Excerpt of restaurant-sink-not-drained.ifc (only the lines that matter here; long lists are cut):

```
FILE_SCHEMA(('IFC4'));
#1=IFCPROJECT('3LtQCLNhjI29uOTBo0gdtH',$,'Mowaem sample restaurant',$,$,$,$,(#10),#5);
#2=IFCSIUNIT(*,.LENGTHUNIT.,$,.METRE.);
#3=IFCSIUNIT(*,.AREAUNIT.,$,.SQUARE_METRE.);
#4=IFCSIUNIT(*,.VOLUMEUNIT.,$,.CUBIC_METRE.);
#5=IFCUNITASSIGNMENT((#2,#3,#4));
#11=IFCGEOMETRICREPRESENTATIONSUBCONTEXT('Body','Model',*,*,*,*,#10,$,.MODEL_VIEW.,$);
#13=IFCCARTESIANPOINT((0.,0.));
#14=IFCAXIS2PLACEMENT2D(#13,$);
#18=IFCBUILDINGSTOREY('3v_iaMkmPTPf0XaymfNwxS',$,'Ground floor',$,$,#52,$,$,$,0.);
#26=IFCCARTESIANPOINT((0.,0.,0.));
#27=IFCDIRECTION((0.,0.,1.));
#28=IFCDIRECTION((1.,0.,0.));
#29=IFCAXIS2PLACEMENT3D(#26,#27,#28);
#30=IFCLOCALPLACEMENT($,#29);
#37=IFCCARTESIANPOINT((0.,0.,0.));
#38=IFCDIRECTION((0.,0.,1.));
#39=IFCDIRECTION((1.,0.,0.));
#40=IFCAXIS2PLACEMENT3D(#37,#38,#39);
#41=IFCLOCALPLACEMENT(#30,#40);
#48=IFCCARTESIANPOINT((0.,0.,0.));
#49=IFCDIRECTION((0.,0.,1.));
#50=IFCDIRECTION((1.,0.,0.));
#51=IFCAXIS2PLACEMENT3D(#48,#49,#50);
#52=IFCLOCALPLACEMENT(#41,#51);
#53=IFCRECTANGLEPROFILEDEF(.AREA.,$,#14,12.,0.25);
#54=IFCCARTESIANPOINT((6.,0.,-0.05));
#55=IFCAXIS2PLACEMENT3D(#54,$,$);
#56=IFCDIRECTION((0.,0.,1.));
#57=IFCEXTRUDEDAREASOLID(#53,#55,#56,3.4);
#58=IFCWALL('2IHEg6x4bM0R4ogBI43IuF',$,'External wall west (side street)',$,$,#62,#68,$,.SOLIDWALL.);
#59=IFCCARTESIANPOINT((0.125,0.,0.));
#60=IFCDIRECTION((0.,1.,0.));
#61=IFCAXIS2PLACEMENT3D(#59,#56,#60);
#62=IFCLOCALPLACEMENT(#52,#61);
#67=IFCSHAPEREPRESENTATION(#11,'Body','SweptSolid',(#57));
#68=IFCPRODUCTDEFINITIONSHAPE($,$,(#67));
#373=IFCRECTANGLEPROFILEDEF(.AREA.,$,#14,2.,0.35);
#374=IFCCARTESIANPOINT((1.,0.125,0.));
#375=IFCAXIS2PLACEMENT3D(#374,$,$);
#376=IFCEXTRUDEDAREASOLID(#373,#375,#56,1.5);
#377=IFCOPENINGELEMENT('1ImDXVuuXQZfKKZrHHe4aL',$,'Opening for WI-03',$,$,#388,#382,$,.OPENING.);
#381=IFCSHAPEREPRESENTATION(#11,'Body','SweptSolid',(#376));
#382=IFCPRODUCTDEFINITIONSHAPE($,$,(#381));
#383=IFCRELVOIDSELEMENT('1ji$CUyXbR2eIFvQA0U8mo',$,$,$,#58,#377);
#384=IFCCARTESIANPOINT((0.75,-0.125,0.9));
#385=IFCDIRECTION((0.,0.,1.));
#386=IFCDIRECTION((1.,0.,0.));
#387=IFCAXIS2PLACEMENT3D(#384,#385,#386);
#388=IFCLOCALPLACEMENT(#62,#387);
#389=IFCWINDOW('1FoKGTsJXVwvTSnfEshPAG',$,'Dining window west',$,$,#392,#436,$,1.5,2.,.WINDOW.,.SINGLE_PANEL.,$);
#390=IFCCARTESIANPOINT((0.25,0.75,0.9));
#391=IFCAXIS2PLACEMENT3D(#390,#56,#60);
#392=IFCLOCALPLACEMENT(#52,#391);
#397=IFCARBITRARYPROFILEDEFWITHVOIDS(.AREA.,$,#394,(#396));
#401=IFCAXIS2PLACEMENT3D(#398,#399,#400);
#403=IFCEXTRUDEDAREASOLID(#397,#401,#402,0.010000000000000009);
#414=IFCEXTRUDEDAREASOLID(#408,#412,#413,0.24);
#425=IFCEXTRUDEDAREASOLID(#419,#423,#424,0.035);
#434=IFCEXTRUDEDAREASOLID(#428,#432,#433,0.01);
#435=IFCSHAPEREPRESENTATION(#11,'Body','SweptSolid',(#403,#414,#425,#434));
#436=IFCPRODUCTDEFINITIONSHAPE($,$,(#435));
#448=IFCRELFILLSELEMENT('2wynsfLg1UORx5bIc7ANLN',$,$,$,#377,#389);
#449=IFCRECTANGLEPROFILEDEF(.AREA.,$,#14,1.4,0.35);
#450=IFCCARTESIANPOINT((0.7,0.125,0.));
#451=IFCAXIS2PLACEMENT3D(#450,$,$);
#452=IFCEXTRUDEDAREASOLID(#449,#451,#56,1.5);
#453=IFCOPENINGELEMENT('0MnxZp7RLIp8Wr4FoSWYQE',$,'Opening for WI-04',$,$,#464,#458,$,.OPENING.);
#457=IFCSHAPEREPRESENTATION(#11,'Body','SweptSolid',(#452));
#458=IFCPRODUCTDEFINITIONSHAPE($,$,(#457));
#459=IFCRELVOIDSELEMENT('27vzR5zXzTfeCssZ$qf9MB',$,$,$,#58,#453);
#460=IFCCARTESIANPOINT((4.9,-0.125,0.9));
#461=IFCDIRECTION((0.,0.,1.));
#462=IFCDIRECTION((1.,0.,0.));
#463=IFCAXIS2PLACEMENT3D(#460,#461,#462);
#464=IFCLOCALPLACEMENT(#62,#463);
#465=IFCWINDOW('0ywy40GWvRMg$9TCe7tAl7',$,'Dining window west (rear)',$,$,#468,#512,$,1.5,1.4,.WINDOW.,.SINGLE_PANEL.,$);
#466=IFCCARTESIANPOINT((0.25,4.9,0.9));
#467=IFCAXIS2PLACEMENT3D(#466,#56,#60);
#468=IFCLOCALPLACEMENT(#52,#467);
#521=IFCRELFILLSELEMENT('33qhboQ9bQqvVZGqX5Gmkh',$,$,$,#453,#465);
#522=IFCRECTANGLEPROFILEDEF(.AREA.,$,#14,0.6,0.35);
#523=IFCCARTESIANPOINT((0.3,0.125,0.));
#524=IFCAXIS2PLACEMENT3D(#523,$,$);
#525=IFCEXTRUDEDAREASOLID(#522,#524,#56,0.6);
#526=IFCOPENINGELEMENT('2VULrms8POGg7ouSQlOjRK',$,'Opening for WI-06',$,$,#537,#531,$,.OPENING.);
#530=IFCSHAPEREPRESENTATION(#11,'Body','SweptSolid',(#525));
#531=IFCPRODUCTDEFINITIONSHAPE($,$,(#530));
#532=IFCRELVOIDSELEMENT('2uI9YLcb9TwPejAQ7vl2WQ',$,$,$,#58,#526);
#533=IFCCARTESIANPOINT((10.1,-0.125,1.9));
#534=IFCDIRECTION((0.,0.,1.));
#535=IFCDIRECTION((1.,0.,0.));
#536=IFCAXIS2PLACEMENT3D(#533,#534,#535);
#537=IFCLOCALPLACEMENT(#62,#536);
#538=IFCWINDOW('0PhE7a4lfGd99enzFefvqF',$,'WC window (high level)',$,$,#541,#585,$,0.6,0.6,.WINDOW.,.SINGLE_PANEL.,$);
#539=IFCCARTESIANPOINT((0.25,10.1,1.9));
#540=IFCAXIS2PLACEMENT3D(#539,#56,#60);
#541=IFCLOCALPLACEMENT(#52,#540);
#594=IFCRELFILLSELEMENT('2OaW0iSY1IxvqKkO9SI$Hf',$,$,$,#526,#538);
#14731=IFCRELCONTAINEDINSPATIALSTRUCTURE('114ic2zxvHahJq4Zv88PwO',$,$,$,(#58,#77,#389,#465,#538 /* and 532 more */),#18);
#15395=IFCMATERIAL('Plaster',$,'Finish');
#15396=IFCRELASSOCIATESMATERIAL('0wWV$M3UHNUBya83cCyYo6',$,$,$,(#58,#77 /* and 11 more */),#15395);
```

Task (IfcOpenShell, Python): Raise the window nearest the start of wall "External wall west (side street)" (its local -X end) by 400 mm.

```python
import numpy as np
import ifcopenshell
import ifcopenshell.api.geometry
import ifcopenshell.util.placement
import ifcopenshell.util.unit

model = ifcopenshell.open("restaurant-sink-not-drained.ifc")
unit_scale = ifcopenshell.util.unit.calculate_unit_scale(model)

window = model.by_id(389)
opening = window.FillsVoids[0].RelatingOpeningElement
dz = 0.4 / unit_scale

shift = np.array([0.0, 0.0, dz])
# The window is not placed relative to its opening, so move both.
for product in (opening, window):
    matrix = ifcopenshell.util.placement.get_local_placement(product.ObjectPlacement)
    matrix[:3, 3] += shift
    ifcopenshell.api.geometry.edit_object_placement(model, product=product, matrix=matrix, is_si=False)

print(f"moved by {dz * unit_scale:+.3f} m")

model.write("restaurant-sink-not-drained_updated.ifc")
```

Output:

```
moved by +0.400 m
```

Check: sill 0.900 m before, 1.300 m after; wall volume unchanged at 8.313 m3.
